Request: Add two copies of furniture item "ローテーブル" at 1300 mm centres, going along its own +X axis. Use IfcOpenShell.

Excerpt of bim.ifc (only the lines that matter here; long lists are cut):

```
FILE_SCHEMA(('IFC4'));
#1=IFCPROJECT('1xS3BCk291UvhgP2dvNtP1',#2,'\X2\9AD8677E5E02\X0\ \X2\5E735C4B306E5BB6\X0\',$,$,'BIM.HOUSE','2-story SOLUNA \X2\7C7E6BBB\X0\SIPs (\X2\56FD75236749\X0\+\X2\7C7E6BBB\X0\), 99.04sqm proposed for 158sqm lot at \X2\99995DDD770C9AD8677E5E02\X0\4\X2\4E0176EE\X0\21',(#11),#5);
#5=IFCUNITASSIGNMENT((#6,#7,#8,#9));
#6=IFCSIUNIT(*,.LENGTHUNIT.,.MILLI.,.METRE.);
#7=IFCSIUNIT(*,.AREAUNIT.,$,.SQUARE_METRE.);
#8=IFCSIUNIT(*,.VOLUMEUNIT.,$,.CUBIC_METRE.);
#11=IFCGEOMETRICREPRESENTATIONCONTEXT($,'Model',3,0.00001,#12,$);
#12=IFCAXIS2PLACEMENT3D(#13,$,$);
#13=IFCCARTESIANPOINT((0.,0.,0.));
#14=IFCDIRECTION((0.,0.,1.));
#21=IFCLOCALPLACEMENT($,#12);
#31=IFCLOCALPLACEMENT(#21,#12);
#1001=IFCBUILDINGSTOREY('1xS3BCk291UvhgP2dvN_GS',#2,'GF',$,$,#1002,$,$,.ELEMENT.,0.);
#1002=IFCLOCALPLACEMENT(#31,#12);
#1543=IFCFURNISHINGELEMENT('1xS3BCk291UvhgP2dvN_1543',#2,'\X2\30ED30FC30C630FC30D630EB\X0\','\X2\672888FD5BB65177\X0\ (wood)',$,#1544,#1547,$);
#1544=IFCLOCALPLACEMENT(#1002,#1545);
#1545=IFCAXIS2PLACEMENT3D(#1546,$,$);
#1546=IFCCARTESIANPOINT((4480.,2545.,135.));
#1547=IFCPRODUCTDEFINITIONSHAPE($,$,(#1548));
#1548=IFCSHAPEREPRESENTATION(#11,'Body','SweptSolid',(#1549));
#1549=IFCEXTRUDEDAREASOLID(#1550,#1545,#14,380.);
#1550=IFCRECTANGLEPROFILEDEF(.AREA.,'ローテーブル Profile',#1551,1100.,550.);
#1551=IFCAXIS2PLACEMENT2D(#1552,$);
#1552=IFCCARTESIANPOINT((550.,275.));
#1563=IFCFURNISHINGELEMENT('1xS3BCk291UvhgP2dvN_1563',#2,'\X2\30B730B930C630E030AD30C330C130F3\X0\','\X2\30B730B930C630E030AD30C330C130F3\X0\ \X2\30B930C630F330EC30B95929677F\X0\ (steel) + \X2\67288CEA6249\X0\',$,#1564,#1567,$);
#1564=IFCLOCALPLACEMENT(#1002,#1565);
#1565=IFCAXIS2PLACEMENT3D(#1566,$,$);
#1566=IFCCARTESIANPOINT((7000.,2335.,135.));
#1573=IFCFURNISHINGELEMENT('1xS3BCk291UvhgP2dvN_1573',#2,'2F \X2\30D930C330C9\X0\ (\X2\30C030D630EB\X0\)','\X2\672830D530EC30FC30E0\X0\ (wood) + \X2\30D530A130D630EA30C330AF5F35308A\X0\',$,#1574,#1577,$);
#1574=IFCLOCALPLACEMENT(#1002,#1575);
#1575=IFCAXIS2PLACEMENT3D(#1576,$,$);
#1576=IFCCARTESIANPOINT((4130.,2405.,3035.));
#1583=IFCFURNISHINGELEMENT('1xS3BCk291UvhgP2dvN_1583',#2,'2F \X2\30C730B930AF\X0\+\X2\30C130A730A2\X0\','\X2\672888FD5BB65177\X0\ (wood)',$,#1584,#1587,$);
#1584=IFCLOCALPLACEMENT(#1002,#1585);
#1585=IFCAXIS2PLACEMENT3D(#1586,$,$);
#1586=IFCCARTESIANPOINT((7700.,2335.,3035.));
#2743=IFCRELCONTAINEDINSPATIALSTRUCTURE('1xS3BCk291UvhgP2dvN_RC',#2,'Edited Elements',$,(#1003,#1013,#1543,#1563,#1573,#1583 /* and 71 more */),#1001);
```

```python
import ifcopenshell
import ifcopenshell.api.geometry
import ifcopenshell.api.root
import ifcopenshell.util.element
import ifcopenshell.util.placement
import ifcopenshell.util.unit

model = ifcopenshell.open("bim.ifc")
unit_scale = ifcopenshell.util.unit.calculate_unit_scale(model)


def reuse_history(source, copy):
    """copy_class also copies each property set's owner history, people and application; keep the originals."""
    for rel in copy.IsDefinedBy:
        if rel.is_a("IfcRelDefinesByProperties") and (history := rel.RelatingPropertyDefinition.OwnerHistory):
            rel.RelatingPropertyDefinition.OwnerHistory = source.OwnerHistory
            ifcopenshell.util.element.remove_deep2(model, history)


source = model.by_guid("1xS3BCk291UvhgP2dvN_1543")
base = ifcopenshell.util.placement.get_local_placement(source.ObjectPlacement)
step = base[:3, 0] * 1.3 / unit_scale

for i in range(1, 3):
    copy = ifcopenshell.api.root.copy_class(model, product=source)
    copy.Representation = ifcopenshell.util.element.copy_deep(
        model, source.Representation, exclude=["IfcGeometricRepresentationContext", "IfcRepresentationMap"]
    )
    reuse_history(source, copy)
    matrix = base.copy()
    matrix[:3, 3] += i * step
    print("added at", matrix[:3, 3].round(3) + 0.0)
    ifcopenshell.api.geometry.edit_object_placement(model, product=copy, matrix=matrix, is_si=False)

model.write("bim_v2.ifc")
```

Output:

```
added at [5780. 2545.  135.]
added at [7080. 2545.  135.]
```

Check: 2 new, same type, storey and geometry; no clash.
